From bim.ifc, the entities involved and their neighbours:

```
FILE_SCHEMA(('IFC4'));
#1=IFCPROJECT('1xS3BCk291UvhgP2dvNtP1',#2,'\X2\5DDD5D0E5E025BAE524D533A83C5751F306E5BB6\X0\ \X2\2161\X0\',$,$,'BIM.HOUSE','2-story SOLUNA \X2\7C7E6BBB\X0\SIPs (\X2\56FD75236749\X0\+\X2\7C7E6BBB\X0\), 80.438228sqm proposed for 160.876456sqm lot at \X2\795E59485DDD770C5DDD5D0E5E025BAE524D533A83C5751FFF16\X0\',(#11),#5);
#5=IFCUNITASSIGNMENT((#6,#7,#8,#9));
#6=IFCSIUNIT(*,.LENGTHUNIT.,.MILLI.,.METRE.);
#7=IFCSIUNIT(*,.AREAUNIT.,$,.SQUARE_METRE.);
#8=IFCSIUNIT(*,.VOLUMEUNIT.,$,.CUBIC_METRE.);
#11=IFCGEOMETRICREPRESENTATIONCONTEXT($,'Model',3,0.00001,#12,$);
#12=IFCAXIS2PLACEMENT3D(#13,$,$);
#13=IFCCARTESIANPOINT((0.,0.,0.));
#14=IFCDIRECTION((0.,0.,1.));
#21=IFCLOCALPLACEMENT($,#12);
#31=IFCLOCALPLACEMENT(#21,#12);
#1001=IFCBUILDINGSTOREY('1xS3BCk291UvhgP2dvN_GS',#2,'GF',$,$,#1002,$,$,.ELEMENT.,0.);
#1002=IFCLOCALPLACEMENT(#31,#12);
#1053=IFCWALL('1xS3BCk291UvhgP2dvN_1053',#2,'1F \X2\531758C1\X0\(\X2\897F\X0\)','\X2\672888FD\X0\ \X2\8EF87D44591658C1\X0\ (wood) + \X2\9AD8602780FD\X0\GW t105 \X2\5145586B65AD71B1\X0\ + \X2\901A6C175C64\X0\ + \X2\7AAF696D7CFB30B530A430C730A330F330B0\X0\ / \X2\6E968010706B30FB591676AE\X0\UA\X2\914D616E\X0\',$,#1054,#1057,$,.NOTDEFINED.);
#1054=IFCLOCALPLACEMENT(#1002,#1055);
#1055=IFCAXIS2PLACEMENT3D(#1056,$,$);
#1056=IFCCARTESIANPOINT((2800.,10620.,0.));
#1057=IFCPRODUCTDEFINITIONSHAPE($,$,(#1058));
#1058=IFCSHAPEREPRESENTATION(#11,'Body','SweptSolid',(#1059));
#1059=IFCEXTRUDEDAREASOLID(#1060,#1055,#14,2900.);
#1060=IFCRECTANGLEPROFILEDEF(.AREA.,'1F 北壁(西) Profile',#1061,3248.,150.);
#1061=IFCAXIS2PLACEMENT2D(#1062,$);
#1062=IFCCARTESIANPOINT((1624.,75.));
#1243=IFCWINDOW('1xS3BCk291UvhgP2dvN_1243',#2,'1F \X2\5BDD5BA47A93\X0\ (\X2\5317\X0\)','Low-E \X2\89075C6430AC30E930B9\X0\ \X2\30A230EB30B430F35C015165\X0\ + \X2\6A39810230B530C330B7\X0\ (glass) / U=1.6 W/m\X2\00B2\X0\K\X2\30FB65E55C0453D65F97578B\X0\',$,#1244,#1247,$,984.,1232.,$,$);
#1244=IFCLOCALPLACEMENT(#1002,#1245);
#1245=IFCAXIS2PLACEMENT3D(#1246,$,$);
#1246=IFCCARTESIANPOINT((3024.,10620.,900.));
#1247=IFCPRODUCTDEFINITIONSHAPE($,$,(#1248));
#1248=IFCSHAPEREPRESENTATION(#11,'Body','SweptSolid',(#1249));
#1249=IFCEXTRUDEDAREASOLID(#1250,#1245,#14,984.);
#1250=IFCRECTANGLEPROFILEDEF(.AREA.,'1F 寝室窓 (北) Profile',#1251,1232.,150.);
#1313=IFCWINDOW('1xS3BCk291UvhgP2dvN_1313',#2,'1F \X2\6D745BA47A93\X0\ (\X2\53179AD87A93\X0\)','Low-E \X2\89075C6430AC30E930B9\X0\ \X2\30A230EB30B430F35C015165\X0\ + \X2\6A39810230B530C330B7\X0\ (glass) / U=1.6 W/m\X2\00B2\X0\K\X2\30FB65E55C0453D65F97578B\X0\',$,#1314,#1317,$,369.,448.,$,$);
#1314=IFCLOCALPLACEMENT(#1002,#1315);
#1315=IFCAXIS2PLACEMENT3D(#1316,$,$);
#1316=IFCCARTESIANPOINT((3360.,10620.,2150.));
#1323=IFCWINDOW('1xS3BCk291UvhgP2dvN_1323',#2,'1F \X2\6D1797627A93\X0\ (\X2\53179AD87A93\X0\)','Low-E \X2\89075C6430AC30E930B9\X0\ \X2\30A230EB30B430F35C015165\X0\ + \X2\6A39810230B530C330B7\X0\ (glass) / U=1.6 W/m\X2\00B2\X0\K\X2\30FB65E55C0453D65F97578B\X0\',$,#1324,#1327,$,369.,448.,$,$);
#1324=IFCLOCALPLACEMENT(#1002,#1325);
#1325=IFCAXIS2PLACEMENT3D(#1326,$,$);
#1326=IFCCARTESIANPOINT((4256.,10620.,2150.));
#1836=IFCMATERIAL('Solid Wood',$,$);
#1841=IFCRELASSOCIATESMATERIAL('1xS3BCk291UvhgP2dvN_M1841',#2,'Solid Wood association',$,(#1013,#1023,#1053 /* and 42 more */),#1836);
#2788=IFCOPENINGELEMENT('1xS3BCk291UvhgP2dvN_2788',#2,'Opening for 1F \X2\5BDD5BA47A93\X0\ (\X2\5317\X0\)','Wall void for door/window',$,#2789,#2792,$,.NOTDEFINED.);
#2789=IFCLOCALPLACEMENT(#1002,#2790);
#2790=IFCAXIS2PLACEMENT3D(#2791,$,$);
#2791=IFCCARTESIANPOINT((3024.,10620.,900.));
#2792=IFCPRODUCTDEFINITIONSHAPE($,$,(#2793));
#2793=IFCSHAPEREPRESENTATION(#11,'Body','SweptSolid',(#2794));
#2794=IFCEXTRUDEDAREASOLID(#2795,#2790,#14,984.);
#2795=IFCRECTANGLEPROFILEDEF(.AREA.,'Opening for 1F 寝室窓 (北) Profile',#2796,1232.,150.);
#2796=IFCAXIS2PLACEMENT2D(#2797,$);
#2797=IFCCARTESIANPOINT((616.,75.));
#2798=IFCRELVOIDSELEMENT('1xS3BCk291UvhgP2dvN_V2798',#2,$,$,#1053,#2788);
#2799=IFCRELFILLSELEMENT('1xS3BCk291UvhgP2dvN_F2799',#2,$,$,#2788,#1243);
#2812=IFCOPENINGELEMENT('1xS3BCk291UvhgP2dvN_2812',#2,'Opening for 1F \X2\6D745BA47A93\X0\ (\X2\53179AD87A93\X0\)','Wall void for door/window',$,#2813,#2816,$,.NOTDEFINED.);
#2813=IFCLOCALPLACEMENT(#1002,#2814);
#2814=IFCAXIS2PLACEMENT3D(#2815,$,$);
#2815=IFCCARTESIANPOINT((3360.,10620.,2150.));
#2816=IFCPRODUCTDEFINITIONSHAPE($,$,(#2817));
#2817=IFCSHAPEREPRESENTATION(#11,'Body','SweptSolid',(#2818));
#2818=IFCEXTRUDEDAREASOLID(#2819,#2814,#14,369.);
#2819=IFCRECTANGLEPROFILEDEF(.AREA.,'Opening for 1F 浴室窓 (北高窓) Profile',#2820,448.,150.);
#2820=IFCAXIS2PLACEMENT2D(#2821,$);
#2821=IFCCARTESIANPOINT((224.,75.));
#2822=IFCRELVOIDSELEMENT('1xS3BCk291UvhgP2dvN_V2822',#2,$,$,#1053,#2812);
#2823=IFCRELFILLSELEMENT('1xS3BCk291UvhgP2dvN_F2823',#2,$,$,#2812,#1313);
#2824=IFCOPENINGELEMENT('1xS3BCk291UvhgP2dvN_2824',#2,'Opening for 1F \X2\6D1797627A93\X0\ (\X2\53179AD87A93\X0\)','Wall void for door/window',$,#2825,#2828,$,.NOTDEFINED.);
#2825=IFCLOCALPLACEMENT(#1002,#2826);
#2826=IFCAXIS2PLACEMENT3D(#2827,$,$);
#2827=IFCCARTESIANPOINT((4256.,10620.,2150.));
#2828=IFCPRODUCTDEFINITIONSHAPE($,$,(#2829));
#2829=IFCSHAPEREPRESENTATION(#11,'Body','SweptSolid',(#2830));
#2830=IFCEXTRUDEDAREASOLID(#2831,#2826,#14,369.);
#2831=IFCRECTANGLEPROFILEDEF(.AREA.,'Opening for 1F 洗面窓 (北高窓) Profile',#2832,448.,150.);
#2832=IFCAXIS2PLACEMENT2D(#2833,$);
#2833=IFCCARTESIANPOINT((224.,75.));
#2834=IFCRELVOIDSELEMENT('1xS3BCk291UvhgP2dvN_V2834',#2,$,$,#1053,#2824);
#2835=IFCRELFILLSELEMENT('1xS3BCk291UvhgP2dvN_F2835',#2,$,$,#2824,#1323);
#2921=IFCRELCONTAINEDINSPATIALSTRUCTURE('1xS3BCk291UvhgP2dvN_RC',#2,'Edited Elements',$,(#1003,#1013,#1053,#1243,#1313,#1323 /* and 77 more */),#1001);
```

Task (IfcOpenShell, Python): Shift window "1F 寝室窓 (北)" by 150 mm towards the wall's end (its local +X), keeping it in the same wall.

```python
import ifcopenshell
import ifcopenshell.api.geometry
import ifcopenshell.util.placement
import ifcopenshell.util.unit

model = ifcopenshell.open("bim.ifc")
unit_scale = ifcopenshell.util.unit.calculate_unit_scale(model)

window = model.by_id(1243)
opening = window.FillsVoids[0].RelatingOpeningElement
wall = opening.VoidsElements[0].RelatingBuildingElement

wall_matrix = ifcopenshell.util.placement.get_local_placement(wall.ObjectPlacement)
shift = wall_matrix[:3, 0] * 0.15 / unit_scale
before = ifcopenshell.util.placement.get_local_placement(window.ObjectPlacement)[:3, 3].copy()

# The window is not placed relative to its opening, so move both.
for product in (opening, window):
    matrix = ifcopenshell.util.placement.get_local_placement(product.ObjectPlacement)
    matrix[:3, 3] += shift
    ifcopenshell.api.geometry.edit_object_placement(model, product=product, matrix=matrix, is_si=False)

after = ifcopenshell.util.placement.get_local_placement(window.ObjectPlacement)[:3, 3]
print("window moved by", (after - before).round(3) + 0.0)

model.write("bim_v2.ifc")
```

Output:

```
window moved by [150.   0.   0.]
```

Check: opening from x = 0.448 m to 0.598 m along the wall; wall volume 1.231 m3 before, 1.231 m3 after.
